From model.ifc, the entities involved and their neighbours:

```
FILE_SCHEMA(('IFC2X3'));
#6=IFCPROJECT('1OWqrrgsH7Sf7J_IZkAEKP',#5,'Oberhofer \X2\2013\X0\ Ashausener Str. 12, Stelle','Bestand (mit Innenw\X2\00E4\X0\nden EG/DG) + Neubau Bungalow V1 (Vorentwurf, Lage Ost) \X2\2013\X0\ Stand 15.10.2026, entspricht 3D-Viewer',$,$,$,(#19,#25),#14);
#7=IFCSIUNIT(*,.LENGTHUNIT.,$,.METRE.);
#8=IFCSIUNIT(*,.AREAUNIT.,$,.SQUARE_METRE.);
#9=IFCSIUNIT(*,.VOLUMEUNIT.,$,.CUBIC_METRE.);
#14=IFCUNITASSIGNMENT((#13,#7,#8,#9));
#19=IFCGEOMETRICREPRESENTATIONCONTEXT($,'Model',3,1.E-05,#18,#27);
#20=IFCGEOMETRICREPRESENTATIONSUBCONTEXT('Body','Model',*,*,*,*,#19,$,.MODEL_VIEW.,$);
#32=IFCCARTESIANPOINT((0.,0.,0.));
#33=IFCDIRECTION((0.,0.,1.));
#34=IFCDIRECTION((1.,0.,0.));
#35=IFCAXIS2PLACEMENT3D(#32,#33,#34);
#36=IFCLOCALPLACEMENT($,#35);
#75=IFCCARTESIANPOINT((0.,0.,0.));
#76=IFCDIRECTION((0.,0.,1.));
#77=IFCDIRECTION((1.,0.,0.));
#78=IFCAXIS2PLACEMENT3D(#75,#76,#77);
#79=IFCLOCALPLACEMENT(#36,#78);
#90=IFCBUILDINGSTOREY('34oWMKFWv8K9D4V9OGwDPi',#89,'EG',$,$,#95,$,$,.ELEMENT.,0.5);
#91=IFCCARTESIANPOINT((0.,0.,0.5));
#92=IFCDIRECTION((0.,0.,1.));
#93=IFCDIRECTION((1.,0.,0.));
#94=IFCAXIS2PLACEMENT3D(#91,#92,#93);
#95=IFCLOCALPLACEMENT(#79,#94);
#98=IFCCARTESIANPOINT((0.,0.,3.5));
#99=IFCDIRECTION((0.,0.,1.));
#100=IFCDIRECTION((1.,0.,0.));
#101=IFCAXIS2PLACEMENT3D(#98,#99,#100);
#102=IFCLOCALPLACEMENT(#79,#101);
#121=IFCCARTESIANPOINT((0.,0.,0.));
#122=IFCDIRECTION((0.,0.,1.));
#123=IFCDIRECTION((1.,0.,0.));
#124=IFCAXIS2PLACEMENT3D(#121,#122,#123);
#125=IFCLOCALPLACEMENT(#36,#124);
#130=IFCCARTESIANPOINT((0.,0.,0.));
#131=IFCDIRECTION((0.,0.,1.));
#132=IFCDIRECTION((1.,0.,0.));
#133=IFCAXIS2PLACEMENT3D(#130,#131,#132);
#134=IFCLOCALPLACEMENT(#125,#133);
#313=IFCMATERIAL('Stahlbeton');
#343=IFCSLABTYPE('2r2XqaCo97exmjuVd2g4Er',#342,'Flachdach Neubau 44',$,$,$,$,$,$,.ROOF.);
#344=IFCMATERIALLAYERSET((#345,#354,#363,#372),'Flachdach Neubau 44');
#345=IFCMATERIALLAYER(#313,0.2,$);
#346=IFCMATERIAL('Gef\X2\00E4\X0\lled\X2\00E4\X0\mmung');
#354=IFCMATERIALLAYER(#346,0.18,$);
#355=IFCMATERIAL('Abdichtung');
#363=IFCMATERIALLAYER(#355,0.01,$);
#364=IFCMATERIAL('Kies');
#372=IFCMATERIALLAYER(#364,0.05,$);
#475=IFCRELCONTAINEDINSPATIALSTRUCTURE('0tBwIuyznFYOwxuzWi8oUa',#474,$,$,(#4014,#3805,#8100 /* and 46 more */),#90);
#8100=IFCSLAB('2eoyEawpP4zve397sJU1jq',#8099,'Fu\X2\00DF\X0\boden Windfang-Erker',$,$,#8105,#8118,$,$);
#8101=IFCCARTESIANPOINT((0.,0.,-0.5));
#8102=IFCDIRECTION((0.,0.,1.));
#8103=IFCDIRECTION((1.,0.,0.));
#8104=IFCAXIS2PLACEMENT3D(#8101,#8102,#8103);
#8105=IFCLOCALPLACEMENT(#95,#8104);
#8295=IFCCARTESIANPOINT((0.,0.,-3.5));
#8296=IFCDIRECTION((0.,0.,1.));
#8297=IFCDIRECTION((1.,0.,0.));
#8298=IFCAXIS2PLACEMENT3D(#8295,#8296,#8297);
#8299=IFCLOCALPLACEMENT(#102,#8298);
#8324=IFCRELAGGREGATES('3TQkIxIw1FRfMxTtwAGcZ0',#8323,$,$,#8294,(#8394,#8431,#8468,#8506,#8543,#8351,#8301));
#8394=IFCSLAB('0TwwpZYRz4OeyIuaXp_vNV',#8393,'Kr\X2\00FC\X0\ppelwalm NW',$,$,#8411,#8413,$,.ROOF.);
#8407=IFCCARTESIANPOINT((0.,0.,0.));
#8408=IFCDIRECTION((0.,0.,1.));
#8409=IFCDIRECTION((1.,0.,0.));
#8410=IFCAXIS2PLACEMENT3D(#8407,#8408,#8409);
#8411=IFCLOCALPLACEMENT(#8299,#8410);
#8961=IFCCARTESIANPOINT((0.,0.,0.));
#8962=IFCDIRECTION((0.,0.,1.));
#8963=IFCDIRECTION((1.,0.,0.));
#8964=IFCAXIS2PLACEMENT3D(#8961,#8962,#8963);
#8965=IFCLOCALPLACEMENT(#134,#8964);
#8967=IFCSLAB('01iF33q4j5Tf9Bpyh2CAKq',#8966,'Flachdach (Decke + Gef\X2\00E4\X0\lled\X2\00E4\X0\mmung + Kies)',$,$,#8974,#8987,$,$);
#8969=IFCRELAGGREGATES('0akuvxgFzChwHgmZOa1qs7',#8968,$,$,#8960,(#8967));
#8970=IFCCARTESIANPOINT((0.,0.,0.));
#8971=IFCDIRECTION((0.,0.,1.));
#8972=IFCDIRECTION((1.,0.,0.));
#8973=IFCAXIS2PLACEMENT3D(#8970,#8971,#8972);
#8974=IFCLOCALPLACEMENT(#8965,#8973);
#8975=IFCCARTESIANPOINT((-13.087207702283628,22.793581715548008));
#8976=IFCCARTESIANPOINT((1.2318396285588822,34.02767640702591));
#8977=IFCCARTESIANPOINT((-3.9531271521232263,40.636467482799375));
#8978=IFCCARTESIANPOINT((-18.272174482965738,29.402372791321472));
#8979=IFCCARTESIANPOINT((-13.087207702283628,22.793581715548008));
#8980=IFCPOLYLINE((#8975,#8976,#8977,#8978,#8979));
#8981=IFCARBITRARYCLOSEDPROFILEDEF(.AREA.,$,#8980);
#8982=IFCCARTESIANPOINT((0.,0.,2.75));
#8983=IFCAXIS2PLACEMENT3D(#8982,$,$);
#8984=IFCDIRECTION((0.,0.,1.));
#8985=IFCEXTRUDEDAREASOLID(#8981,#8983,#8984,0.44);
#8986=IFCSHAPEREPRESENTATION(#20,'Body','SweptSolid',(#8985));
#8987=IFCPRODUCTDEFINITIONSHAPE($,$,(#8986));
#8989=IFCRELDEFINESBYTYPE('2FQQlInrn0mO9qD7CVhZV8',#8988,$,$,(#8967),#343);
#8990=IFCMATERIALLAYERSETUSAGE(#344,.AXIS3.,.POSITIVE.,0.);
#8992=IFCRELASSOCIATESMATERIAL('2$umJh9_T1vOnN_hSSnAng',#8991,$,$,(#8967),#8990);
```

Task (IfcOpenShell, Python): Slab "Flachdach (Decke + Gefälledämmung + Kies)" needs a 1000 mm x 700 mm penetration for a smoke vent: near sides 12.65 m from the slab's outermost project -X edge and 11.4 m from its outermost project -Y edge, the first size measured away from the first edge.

```python
import numpy as np
import ifcopenshell
import ifcopenshell.api.feature
import ifcopenshell.api.geometry
import ifcopenshell.api.root
import ifcopenshell.geom
import ifcopenshell.util.placement
import ifcopenshell.util.representation
import ifcopenshell.util.shape
import ifcopenshell.util.unit

model = ifcopenshell.open("model.ifc")
unit_scale = ifcopenshell.util.unit.calculate_unit_scale(model)
settings = ifcopenshell.geom.settings()


def volume(element):
    """Net volume in cubic metres, openings subtracted."""
    shape = ifcopenshell.geom.create_shape(settings, element)
    return ifcopenshell.util.shape.get_volume(shape.geometry)


slab = model.by_guid("01iF33q4j5Tf9Bpyh2CAKq")
before = volume(slab)

# Extent in the slab's own axes, in metres. The edges named are its -X and -Y sides.
slab_shape = ifcopenshell.geom.create_shape(settings, slab)
vertices = ifcopenshell.util.shape.get_vertices(slab_shape.geometry)
x_min, y_min, bottom = vertices.min(axis=0)
top = vertices[:, 2].max()

opening = ifcopenshell.api.root.create_entity(model, ifc_class="IfcOpeningElement", name="Smoke vent opening")
context = ifcopenshell.util.representation.get_context(model, "Model", "Body", "MODEL_VIEW")
width, depth = 1, 0.7
outline = [(0.0, 0.0), (width, 0.0), (width, depth), (0.0, depth), (0.0, 0.0)]
# Overshoot both faces by 50 mm so the cut is clean.
shape = ifcopenshell.api.geometry.add_slab_representation(
    model, context=context, depth=top - bottom + 0.1, polyline=outline
)
ifcopenshell.api.geometry.assign_representation(model, product=opening, representation=shape)

matrix = ifcopenshell.util.placement.get_local_placement(slab.ObjectPlacement)
matrix[:, 3] = matrix @ np.append(np.array([x_min + 12.65, y_min + 11.4, bottom - 0.05]) / unit_scale, 1.0)
ifcopenshell.api.geometry.edit_object_placement(model, product=opening, matrix=matrix, is_si=False)
ifcopenshell.api.feature.add_feature(model, feature=opening, element=slab)

after = volume(slab)

print(f"slab volume {before:.3f} -> {after:.3f} m3")

model.write("model-out.ifc")
```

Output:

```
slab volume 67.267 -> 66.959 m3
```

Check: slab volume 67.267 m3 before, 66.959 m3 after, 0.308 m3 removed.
